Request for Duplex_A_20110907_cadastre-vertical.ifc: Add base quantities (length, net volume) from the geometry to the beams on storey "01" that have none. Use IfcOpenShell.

First a look at what the model holds.

```python
import ifcopenshell
import ifcopenshell.util.element
import ifcopenshell.util.unit

model = ifcopenshell.open("Duplex_A_20110907_cadastre-vertical.ifc")
print(model.schema)
for unit_type in ("LENGTHUNIT", "AREAUNIT", "VOLUMEUNIT"):
    print(unit_type, ifcopenshell.util.unit.calculate_unit_scale(model, unit_type))
storey = next(s for s in model.by_type("IfcBuildingStorey") if s.Name == "01")
beams = [e for e in ifcopenshell.util.element.get_decomposition(storey) if e.is_a("IfcBeam")]
for e in sorted(beams, key=lambda e: e.id()):
    print(e.id(), e.is_a(), e.Name, list(ifcopenshell.util.element.get_psets(e, qtos_only=True)), sep=" | ")
```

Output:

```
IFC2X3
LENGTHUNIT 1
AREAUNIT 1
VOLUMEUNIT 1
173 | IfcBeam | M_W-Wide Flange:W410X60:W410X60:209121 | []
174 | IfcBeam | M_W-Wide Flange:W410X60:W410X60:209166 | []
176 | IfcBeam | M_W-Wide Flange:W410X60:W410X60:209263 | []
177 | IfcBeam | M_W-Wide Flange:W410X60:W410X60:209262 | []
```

```python
import ifcopenshell
import ifcopenshell.api.pset
import ifcopenshell.geom
import ifcopenshell.util.element
import ifcopenshell.util.shape
import ifcopenshell.util.unit

model = ifcopenshell.open("Duplex_A_20110907_cadastre-vertical.ifc")
unit_scale = ifcopenshell.util.unit.calculate_unit_scale(model)
volume_scale = ifcopenshell.util.unit.calculate_unit_scale(model, "VOLUMEUNIT")
settings = ifcopenshell.geom.settings()

storey = next(s for s in model.by_type("IfcBuildingStorey") if s.Name == "01")
beams = [e for e in ifcopenshell.util.element.get_decomposition(storey) if e.is_a("IfcBeam")]

for e in sorted(beams, key=lambda e: e.id()):
    if ifcopenshell.util.element.get_psets(e, qtos_only=True, should_inherit=False):
        continue
    # Geometry comes back in metres, in the element's own axes.
    shape = ifcopenshell.geom.create_shape(settings, e)
    values = {
        "Length": ifcopenshell.util.shape.get_max_xyz(shape.geometry) / unit_scale,
        "NetVolume": ifcopenshell.util.shape.get_volume(shape.geometry) / volume_scale,
    }
    qto = ifcopenshell.api.pset.add_qto(model, product=e, name="BaseQuantities")
    ifcopenshell.api.pset.edit_qto(model, qto=qto, properties=values)
    print(e.id(), {k: round(v, 3) for k, v in values.items()})

model.write("Duplex_A_20110907_cadastre-vertical-out.ifc")
```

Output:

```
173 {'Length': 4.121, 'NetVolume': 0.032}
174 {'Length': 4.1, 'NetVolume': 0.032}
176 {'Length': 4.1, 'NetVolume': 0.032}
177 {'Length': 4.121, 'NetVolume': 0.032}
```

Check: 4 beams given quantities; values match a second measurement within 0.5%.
